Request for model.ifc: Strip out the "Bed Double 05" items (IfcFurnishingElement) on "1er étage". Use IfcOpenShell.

First a look at what the model holds.

```python
import ifcopenshell
import ifcopenshell.util.element

model = ifcopenshell.open("model.ifc")
print(model.schema)
storey = next(s for s in model.by_type("IfcBuildingStorey") if s.Name == "1er étage")
furniture = [e for e in ifcopenshell.util.element.get_decomposition(storey) if e.is_a("IfcFurnishingElement")]
seen = {}
for e in furniture:
    element_type = ifcopenshell.util.element.get_type(e)
    name = element_type.Name if element_type not in (None, e) else None
    seen[name] = seen.get(name, 0) + 1
for name, count in sorted(seen.items(), key=str):
    print(count, "x", name)
```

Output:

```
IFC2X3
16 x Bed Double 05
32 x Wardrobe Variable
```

```python
import ifcopenshell
import ifcopenshell.api.root
import ifcopenshell.util.element

model = ifcopenshell.open("model.ifc")

storey = next(s for s in model.by_type("IfcBuildingStorey") if s.Name == "1er étage")
furniture = [e for e in ifcopenshell.util.element.get_decomposition(storey) if e.is_a("IfcFurnishingElement")]
targets = [e for e in furniture if (t := ifcopenshell.util.element.get_type(e)) not in (None, e) and t.Name == "Bed Double 05"]

for e in targets:
    ifcopenshell.api.root.remove_product(model, product=e)
print(len(targets), "removed")

model.write("model-out.ifc")
```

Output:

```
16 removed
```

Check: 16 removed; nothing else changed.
